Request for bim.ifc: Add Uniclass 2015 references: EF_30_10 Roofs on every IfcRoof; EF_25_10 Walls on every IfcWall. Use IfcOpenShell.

First a look at what the model holds.

```python
import ifcopenshell

model = ifcopenshell.open("bim.ifc")
print(model.schema)
print("classifications:", [c.Name for c in model.by_type("IfcClassification")])
for ifc_class in ("IfcDoor", "IfcRoof", "IfcStair", "IfcWall", "IfcWindow"):
    print(ifc_class, len(model.by_type(ifc_class)))
```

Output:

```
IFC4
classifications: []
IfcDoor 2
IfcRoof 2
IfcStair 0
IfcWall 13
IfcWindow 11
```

```python
import ifcopenshell
import ifcopenshell.api.classification

model = ifcopenshell.open("bim.ifc")

system = ifcopenshell.api.classification.add_classification(model, classification="Uniclass 2015")

codes = {
    "IfcRoof": ("EF_30_10", "Roofs"),
    "IfcWall": ("EF_25_10", "Walls"),
}
for ifc_class, (code, name) in codes.items():
    products = model.by_type(ifc_class)
    ifcopenshell.api.classification.add_reference(
        model, products=products, classification=system, identification=code, name=name
    )
    print(code, len(products))

model.write("bim_updated.ifc")
```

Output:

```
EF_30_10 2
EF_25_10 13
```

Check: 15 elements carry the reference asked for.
